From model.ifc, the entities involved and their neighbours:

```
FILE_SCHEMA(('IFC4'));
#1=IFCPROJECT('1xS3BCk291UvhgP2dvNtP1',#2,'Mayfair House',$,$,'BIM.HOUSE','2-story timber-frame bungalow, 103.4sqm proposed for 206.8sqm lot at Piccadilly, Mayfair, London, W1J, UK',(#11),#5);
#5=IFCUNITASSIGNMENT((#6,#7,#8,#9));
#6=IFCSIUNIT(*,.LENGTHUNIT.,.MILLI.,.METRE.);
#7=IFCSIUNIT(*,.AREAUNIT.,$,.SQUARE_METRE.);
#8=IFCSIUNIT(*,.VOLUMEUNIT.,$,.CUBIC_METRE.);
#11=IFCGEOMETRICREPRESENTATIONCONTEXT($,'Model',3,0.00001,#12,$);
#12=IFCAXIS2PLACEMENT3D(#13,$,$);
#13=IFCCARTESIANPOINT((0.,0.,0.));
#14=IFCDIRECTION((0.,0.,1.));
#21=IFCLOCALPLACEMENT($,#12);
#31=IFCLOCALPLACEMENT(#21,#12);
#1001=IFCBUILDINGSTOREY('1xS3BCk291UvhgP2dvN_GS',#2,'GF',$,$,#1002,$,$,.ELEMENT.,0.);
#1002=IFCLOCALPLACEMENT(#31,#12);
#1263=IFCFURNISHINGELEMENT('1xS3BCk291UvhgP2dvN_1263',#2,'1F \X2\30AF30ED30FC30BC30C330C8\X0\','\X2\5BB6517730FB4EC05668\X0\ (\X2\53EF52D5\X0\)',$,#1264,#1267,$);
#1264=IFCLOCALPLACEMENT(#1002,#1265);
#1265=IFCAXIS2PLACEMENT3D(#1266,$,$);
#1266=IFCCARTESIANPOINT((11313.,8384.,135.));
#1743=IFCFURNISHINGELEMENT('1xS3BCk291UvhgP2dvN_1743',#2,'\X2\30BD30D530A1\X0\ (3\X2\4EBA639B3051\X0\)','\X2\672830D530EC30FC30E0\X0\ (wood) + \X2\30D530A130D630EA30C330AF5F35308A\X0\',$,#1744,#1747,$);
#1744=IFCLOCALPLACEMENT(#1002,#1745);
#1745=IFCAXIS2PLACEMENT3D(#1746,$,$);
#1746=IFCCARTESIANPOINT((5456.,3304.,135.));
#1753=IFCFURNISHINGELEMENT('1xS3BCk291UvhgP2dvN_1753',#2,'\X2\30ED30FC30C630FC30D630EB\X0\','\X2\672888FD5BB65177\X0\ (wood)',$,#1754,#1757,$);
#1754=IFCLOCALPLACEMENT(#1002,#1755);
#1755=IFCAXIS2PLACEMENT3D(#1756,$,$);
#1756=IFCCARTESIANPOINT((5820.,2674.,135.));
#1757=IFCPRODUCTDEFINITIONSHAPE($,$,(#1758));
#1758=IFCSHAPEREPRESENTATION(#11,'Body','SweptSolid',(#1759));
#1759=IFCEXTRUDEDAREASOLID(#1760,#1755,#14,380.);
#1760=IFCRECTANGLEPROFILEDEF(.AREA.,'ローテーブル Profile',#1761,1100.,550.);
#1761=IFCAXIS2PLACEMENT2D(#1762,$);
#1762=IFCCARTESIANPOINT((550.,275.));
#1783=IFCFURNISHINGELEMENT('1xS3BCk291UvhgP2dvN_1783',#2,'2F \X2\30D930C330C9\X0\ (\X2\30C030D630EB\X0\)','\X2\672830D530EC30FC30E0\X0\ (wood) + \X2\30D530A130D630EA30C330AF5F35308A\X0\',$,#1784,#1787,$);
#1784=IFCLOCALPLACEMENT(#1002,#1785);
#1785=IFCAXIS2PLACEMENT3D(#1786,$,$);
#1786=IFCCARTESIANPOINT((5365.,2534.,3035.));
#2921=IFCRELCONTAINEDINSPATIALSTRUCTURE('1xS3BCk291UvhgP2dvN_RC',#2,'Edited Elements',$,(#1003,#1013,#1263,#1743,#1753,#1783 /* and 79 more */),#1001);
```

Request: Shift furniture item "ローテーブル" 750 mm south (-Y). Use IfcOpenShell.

```python
import ifcopenshell
import ifcopenshell.api.geometry
import ifcopenshell.util.placement

model = ifcopenshell.open("model.ifc")

item = model.by_id(1753)
matrix = ifcopenshell.util.placement.get_local_placement(item.ObjectPlacement)
matrix[1, 3] -= 750.0
ifcopenshell.api.geometry.edit_object_placement(model, product=item, matrix=matrix, is_si=False)

print(ifcopenshell.util.placement.get_local_placement(item.ObjectPlacement).round(3) + 0.0)

model.write("model_v2.ifc")
```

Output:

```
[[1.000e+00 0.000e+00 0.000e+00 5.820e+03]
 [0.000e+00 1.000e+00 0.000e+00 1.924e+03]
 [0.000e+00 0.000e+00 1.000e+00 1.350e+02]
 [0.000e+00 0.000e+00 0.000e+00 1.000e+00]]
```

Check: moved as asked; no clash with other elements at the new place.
